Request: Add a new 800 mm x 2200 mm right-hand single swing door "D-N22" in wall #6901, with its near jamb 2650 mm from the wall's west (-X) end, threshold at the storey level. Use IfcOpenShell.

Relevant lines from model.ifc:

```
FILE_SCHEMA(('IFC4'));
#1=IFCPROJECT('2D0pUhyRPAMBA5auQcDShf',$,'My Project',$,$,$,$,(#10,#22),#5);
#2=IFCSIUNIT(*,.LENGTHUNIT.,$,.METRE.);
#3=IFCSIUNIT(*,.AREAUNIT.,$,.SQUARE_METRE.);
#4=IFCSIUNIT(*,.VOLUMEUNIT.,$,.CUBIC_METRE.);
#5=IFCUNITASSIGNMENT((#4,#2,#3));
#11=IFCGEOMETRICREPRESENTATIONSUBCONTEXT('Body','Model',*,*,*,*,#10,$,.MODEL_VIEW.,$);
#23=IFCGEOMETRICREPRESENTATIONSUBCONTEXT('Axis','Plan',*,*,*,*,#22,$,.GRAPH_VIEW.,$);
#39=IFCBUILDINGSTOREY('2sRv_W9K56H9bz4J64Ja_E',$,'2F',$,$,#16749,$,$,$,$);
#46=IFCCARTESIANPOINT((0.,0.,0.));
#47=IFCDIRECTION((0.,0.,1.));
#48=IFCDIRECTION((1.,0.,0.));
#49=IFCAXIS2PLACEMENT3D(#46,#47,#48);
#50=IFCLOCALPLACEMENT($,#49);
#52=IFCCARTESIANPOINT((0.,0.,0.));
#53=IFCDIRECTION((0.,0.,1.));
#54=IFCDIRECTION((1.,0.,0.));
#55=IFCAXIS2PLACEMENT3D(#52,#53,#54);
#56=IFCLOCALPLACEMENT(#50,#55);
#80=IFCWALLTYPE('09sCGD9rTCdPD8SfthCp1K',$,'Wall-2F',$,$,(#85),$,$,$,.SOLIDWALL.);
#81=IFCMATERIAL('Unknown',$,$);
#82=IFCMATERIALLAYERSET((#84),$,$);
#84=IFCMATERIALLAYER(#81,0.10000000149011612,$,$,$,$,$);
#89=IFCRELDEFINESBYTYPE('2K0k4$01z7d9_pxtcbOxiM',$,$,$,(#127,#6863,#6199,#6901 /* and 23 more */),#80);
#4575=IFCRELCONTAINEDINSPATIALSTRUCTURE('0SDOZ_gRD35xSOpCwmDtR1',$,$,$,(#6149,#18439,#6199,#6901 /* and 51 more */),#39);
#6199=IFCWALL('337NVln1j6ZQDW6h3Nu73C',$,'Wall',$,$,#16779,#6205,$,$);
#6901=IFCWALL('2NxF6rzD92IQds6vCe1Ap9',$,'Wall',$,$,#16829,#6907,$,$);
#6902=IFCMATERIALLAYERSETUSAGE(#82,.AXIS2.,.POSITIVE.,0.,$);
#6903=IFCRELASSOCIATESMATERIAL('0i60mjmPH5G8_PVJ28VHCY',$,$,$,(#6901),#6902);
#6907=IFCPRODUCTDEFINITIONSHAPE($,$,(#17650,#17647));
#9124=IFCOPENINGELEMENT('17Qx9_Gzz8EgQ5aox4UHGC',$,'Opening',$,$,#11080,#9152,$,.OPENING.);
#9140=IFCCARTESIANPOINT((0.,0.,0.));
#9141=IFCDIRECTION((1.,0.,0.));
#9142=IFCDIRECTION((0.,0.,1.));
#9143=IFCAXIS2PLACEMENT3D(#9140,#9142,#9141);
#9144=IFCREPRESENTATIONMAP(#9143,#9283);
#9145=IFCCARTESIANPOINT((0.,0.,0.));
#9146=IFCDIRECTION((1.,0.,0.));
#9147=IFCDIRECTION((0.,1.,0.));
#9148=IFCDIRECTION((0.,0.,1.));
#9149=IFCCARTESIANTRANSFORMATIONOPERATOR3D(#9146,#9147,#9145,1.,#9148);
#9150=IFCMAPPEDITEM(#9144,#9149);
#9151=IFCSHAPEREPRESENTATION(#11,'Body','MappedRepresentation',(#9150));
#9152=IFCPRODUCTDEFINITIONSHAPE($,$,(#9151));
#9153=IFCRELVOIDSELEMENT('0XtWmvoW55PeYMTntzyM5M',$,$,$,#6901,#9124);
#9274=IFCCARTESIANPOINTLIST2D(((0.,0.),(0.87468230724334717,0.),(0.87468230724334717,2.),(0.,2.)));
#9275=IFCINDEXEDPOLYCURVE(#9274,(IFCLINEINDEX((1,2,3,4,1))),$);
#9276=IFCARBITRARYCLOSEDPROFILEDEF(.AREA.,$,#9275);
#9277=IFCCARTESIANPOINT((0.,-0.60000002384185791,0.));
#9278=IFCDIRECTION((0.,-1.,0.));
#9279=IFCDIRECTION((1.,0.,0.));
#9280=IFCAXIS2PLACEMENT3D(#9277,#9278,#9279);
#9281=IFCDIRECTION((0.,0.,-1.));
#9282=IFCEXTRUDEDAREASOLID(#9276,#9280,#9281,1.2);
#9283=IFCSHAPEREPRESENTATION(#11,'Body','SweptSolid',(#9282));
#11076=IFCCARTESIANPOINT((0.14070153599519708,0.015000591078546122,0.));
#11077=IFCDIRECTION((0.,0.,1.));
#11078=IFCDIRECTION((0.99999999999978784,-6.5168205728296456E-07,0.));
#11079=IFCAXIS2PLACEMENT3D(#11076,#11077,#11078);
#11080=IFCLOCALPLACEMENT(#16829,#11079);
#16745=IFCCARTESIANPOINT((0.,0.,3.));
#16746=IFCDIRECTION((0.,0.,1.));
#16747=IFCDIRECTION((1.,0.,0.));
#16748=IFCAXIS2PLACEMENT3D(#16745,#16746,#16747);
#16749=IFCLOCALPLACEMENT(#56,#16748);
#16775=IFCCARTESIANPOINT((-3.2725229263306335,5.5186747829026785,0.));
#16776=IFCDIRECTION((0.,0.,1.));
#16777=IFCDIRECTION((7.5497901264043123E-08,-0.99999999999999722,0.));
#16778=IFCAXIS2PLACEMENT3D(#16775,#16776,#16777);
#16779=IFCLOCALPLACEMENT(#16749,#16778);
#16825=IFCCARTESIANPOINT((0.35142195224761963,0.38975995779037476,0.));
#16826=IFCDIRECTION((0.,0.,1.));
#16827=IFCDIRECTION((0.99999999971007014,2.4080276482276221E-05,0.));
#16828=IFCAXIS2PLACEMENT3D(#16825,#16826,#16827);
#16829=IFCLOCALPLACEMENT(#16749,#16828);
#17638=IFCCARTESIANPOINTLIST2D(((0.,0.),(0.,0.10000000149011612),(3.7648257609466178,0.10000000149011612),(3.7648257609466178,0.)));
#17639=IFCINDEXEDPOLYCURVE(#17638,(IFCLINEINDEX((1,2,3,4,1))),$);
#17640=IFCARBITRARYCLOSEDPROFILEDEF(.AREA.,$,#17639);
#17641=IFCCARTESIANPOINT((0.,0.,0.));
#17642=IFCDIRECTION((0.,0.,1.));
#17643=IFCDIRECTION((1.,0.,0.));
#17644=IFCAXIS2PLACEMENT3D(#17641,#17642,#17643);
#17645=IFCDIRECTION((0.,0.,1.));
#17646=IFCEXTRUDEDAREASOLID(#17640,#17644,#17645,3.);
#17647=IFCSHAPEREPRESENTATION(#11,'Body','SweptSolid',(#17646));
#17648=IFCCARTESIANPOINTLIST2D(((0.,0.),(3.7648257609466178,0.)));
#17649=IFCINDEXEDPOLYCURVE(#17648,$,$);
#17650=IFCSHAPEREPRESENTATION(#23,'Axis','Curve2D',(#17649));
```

```python
import numpy as np
import ifcopenshell
import ifcopenshell.api.feature
import ifcopenshell.api.geometry
import ifcopenshell.api.root
import ifcopenshell.api.spatial
import ifcopenshell.geom
import ifcopenshell.util.element
import ifcopenshell.util.placement
import ifcopenshell.util.representation
import ifcopenshell.util.shape
import ifcopenshell.util.unit

model = ifcopenshell.open("model.ifc")
unit_scale = ifcopenshell.util.unit.calculate_unit_scale(model)
settings = ifcopenshell.geom.settings()


def volume(element):
    """Net volume in cubic metres, openings subtracted."""
    shape = ifcopenshell.geom.create_shape(settings, element)
    return ifcopenshell.util.shape.get_volume(shape.geometry)


wall = model.by_id(6901)
storey = ifcopenshell.util.element.get_container(wall, ifc_class="IfcBuildingStorey")
context = ifcopenshell.util.representation.get_context(model, "Model", "Body", "MODEL_VIEW")
before = volume(wall)

width, height, from_end, sill = 0.8, 2.2, 2.65, 0.0  # metres

# The wall runs along its own X axis, and the end named is its -X end.
wall_shape = ifcopenshell.geom.create_shape(settings, wall)
x, y, z = ifcopenshell.util.shape.get_vertices(wall_shape.geometry).T
start = x.min() + from_end
face, thickness = float(y.min()), float(y.max() - y.min())
wall_matrix = ifcopenshell.util.placement.get_local_placement(wall.ObjectPlacement)
level = ifcopenshell.util.placement.get_local_placement(storey.ObjectPlacement)[2, 3]


def in_wall(x, y):
    """Placement at x, y metres in the wall's axes, at sill height."""
    matrix = wall_matrix.copy()
    matrix[:, 3] = wall_matrix @ np.array([x / unit_scale, y / unit_scale, 0.0, 1.0])
    matrix[2, 3] = level + sill / unit_scale
    return matrix


# Opening: a box that overshoots both wall faces by 50 mm.
opening = ifcopenshell.api.root.create_entity(model, ifc_class="IfcOpeningElement", predefined_type="OPENING")
box = ifcopenshell.api.geometry.add_wall_representation(
    model, context=context, length=width, height=height, thickness=thickness + 0.1
)
ifcopenshell.api.geometry.assign_representation(model, product=opening, representation=box)
ifcopenshell.api.geometry.edit_object_placement(model, product=opening, matrix=in_wall(start, face - 0.05), is_si=False)
ifcopenshell.api.feature.add_feature(model, feature=opening, element=wall)

door = ifcopenshell.api.root.create_entity(model, ifc_class="IfcDoor", name="D-N22", predefined_type="DOOR")
door.OverallWidth, door.OverallHeight = width / unit_scale, height / unit_scale
door.OperationType = "SINGLE_SWING_RIGHT"
body = ifcopenshell.api.geometry.add_door_representation(
    model,
    context=context,
    overall_width=door.OverallWidth,
    overall_height=door.OverallHeight,
    operation_type="SINGLE_SWING_RIGHT",
    lining_properties={"LiningDepth": thickness / unit_scale, "ThresholdDepth": thickness / unit_scale},
)
ifcopenshell.api.geometry.assign_representation(model, product=door, representation=body)
ifcopenshell.api.spatial.assign_container(model, products=[door], relating_structure=storey)
ifcopenshell.api.feature.add_filling(model, opening=opening, element=door)

# The lining spans the wall, so the door starts at the wall face.
ifcopenshell.api.geometry.edit_object_placement(model, product=door, matrix=in_wall(start, face), is_si=False)

after = volume(wall)

print(f"wall volume {before:.3f} -> {after:.3f} m3")

model.write("model_v2.ifc")
```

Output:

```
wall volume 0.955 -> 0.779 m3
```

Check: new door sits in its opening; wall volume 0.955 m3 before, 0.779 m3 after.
